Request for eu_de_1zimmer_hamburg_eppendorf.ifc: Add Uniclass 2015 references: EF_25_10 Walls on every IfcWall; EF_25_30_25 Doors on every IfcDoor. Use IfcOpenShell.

First a look at what the model holds.

```python
import ifcopenshell

model = ifcopenshell.open("eu_de_1zimmer_hamburg_eppendorf.ifc")
print(model.schema)
print("classifications:", [c.Name for c in model.by_type("IfcClassification")])
for ifc_class in ("IfcDoor", "IfcRoof", "IfcStair", "IfcWall", "IfcWindow"):
    print(ifc_class, len(model.by_type(ifc_class)))
```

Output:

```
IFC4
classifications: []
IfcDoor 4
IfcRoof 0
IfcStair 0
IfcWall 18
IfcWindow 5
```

```python
import ifcopenshell
import ifcopenshell.api.classification

model = ifcopenshell.open("eu_de_1zimmer_hamburg_eppendorf.ifc")

system = ifcopenshell.api.classification.add_classification(model, classification="Uniclass 2015")

codes = {
    "IfcWall": ("EF_25_10", "Walls"),
    "IfcDoor": ("EF_25_30_25", "Doors"),
}
for ifc_class, (code, name) in codes.items():
    products = model.by_type(ifc_class)
    ifcopenshell.api.classification.add_reference(
        model, products=products, classification=system, identification=code, name=name
    )
    print(code, len(products))

model.write("eu_de_1zimmer_hamburg_eppendorf_rev.ifc")
```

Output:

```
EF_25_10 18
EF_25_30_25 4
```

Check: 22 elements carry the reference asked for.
